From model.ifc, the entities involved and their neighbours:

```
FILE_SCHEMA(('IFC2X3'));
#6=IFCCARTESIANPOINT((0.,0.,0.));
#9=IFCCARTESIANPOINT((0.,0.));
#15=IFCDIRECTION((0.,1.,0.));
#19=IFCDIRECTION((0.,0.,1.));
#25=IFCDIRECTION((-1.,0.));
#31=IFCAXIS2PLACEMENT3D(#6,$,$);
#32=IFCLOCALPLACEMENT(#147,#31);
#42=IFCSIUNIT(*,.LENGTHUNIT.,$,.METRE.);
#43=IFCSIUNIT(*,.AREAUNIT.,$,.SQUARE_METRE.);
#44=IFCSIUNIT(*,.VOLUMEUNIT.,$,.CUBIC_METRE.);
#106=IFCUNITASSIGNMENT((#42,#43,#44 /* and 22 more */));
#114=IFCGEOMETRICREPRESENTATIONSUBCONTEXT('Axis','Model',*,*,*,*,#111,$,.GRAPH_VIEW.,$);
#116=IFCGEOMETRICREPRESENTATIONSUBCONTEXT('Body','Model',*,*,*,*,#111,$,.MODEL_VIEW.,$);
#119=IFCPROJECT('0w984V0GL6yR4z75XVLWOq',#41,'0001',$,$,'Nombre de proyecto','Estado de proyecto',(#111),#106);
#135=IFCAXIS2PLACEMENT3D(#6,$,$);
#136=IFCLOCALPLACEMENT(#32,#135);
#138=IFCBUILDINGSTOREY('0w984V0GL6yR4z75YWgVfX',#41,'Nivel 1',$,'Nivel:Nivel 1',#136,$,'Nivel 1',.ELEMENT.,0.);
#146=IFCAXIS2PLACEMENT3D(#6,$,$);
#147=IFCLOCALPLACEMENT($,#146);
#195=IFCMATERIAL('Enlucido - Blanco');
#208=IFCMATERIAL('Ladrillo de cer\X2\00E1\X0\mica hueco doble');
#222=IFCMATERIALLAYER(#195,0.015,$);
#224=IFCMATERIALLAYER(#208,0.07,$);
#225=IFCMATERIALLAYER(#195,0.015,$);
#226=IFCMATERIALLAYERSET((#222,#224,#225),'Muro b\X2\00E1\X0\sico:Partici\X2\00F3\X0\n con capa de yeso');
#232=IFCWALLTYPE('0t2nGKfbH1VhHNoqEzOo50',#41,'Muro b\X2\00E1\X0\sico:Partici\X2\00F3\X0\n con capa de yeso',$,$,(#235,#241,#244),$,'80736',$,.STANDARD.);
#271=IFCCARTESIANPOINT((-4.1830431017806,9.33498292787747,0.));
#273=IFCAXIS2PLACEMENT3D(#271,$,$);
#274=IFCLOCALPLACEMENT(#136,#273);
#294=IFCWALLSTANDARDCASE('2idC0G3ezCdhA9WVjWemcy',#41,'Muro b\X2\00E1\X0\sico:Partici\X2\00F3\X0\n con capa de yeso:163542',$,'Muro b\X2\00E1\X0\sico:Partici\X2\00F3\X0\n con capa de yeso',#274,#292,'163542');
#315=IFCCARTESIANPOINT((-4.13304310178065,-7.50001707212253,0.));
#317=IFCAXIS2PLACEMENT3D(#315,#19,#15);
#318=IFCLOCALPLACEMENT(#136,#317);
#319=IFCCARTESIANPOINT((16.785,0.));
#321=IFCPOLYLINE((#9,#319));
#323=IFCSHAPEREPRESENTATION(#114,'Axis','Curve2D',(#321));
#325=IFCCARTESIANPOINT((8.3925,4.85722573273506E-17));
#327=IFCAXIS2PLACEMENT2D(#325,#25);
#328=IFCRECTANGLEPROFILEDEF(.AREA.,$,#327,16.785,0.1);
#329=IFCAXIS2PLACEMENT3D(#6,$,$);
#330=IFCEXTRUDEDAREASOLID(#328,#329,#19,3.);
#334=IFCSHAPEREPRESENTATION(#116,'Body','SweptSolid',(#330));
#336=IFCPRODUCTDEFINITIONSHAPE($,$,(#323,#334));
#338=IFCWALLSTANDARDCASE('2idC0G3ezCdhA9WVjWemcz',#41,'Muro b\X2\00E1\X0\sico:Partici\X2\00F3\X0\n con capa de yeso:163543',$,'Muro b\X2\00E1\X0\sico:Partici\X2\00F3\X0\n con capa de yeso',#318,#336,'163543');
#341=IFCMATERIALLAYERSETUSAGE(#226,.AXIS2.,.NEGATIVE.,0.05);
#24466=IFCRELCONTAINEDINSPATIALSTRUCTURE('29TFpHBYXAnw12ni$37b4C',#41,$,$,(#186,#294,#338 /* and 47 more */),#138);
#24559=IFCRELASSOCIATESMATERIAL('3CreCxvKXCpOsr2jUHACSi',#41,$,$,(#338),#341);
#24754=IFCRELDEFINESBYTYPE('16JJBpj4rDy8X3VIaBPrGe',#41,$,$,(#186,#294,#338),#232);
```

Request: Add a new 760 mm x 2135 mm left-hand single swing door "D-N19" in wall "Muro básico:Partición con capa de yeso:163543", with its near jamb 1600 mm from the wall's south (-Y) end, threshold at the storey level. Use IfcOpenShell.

```python
import numpy as np
import ifcopenshell
import ifcopenshell.api.feature
import ifcopenshell.api.geometry
import ifcopenshell.api.root
import ifcopenshell.api.spatial
import ifcopenshell.api.type
import ifcopenshell.geom
import ifcopenshell.util.element
import ifcopenshell.util.placement
import ifcopenshell.util.representation
import ifcopenshell.util.shape
import ifcopenshell.util.unit

model = ifcopenshell.open("model.ifc")
unit_scale = ifcopenshell.util.unit.calculate_unit_scale(model)
settings = ifcopenshell.geom.settings()


def volume(element):
    """Net volume in cubic metres, openings subtracted."""
    shape = ifcopenshell.geom.create_shape(settings, element)
    return ifcopenshell.util.shape.get_volume(shape.geometry)


wall = model.by_guid("2idC0G3ezCdhA9WVjWemcz")
storey = ifcopenshell.util.element.get_container(wall, ifc_class="IfcBuildingStorey")
context = ifcopenshell.util.representation.get_context(model, "Model", "Body", "MODEL_VIEW")
before = volume(wall)

width, height, from_end, sill = 0.76, 2.135, 1.6, 0.0  # metres

# The wall runs along its own X axis, and the end named is its -X end.
wall_shape = ifcopenshell.geom.create_shape(settings, wall)
x, y, z = ifcopenshell.util.shape.get_vertices(wall_shape.geometry).T
start = x.min() + from_end
face, thickness = float(y.min()), float(y.max() - y.min())
wall_matrix = ifcopenshell.util.placement.get_local_placement(wall.ObjectPlacement)
level = ifcopenshell.util.placement.get_local_placement(storey.ObjectPlacement)[2, 3]


def in_wall(x, y):
    """Placement at x, y metres in the wall's axes, at sill height."""
    matrix = wall_matrix.copy()
    matrix[:, 3] = wall_matrix @ np.array([x / unit_scale, y / unit_scale, 0.0, 1.0])
    matrix[2, 3] = level + sill / unit_scale
    return matrix


# Opening: a box that overshoots both wall faces by 50 mm.
opening = ifcopenshell.api.root.create_entity(model, ifc_class="IfcOpeningElement")
box = ifcopenshell.api.geometry.add_wall_representation(
    model, context=context, length=width, height=height, thickness=thickness + 0.1
)
ifcopenshell.api.geometry.assign_representation(model, product=opening, representation=box)
ifcopenshell.api.geometry.edit_object_placement(model, product=opening, matrix=in_wall(start, face - 0.05), is_si=False)
ifcopenshell.api.feature.add_feature(model, feature=opening, element=wall)

door = ifcopenshell.api.root.create_entity(model, ifc_class="IfcDoor", name="D-N19")
door.OverallWidth, door.OverallHeight = width / unit_scale, height / unit_scale
body = ifcopenshell.api.geometry.add_door_representation(
    model,
    context=context,
    overall_width=door.OverallWidth,
    overall_height=door.OverallHeight,
    operation_type="SINGLE_SWING_LEFT",
    lining_properties={"LiningDepth": thickness / unit_scale, "ThresholdDepth": thickness / unit_scale},
)
ifcopenshell.api.geometry.assign_representation(model, product=door, representation=body)
ifcopenshell.api.spatial.assign_container(model, products=[door], relating_structure=storey)
fills = ifcopenshell.api.feature.add_filling(model, opening=opening, element=door)
fills.OwnerHistory = door.OwnerHistory  # required in IFC2X3

# IFC2X3 keeps the operation on the door style.
style = ifcopenshell.api.root.create_entity(model, ifc_class="IfcDoorStyle", name="D-N19")
style.OperationType, style.ConstructionType = "SINGLE_SWING_LEFT", "NOTDEFINED"
style.ParameterTakesPrecedence = style.Sizeable = False
ifcopenshell.api.type.assign_type(model, related_objects=[door], relating_type=style)

# The lining spans the wall, so the door starts at the wall face.
ifcopenshell.api.geometry.edit_object_placement(model, product=door, matrix=in_wall(start, face), is_si=False)

after = volume(wall)

print(f"wall volume {before:.3f} -> {after:.3f} m3")

model.write("model_v2.ifc")
```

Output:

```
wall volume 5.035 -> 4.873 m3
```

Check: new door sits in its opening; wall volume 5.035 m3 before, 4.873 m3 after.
